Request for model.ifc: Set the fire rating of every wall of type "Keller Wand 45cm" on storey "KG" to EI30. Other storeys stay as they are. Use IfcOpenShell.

First a look at what the model holds.

```python
import ifcopenshell
import ifcopenshell.util.element

model = ifcopenshell.open("model.ifc")
print(model.schema)
storey = next(s for s in model.by_type("IfcBuildingStorey") if s.Name == "KG")
walls = [e for e in ifcopenshell.util.element.get_decomposition(storey) if e.is_a("IfcWall")]
seen = {}
for e in walls:
    element_type = ifcopenshell.util.element.get_type(e)
    key = (element_type.Name if element_type != e and element_type else None, ifcopenshell.util.element.get_pset(e, "Pset_WallCommon", "FireRating"))
    seen[key] = seen.get(key, 0) + 1
for (name, value), count in sorted(seen.items(), key=str):
    print(count, "x", name, "|", value)
```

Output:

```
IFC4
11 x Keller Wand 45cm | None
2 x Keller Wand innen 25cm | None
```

```python
import ifcopenshell
import ifcopenshell.api.pset
import ifcopenshell.util.element

model = ifcopenshell.open("model.ifc")

storey = next(s for s in model.by_type("IfcBuildingStorey") if s.Name == "KG")
walls = [e for e in ifcopenshell.util.element.get_decomposition(storey) if e.is_a("IfcWall")]

count = 0
for e in walls:
    element_type = ifcopenshell.util.element.get_type(e)
    if element_type in (None, e) or element_type.Name != "Keller Wand 45cm":
        continue
    # add_pset returns the element's existing set when there is one.
    pset = ifcopenshell.api.pset.add_pset(model, product=e, name="Pset_WallCommon")
    ifcopenshell.api.pset.edit_pset(model, pset=pset, properties={"FireRating": "EI30"})
    count += 1

print(count, "walls updated")

model.write("model_v2.ifc")
```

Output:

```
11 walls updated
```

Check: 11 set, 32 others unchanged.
